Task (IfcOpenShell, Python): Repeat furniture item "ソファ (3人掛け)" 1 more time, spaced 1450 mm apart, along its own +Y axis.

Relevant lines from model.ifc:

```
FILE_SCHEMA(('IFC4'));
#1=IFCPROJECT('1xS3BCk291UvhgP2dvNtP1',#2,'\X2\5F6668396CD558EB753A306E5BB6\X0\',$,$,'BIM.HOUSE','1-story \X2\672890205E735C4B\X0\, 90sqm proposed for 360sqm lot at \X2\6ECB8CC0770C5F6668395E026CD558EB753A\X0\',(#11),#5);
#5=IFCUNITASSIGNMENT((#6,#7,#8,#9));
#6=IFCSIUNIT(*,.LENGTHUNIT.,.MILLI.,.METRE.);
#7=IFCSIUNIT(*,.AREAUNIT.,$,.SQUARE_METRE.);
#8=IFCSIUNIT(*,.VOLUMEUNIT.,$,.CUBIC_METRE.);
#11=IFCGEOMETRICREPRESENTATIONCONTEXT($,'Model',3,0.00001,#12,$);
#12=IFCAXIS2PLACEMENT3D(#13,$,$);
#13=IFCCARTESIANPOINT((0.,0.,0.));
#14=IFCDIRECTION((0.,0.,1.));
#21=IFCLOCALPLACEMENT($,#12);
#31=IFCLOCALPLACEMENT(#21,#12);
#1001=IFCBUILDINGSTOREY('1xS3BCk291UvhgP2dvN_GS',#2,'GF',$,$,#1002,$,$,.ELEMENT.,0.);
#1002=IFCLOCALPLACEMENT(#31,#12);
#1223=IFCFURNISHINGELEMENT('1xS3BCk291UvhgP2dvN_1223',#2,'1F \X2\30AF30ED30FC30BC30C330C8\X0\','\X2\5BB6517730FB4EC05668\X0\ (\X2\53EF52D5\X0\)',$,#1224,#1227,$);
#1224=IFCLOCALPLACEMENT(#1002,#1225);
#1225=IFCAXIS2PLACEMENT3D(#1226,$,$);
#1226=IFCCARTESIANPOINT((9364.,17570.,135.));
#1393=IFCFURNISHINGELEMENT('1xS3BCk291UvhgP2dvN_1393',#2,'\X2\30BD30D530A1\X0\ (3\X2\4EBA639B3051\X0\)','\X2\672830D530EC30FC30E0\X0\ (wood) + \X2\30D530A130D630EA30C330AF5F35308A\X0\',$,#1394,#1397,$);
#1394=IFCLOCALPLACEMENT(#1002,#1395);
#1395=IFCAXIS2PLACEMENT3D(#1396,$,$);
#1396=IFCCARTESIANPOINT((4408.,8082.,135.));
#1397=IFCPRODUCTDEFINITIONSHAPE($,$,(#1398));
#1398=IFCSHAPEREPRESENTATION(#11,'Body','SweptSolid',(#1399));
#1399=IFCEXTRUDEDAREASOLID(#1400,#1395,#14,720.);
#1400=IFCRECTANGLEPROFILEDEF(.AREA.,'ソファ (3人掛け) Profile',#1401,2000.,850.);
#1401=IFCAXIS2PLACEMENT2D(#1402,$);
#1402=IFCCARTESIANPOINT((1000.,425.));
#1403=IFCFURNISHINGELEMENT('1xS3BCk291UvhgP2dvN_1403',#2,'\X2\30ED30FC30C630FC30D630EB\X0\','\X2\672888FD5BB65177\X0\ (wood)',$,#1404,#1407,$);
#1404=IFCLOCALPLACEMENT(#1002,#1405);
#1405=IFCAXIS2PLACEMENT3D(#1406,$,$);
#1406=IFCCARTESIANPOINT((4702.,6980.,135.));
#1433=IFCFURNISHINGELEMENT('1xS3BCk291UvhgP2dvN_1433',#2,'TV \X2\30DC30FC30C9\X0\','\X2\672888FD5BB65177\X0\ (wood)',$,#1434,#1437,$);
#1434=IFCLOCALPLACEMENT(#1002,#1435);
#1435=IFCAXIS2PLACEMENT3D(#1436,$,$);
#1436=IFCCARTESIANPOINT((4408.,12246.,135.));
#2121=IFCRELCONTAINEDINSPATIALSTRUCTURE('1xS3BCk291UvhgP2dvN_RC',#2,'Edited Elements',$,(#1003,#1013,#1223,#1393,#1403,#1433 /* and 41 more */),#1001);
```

```python
import ifcopenshell
import ifcopenshell.api.geometry
import ifcopenshell.api.root
import ifcopenshell.util.element
import ifcopenshell.util.placement
import ifcopenshell.util.unit

model = ifcopenshell.open("model.ifc")
unit_scale = ifcopenshell.util.unit.calculate_unit_scale(model)


def reuse_history(source, copy):
    """copy_class also copies each property set's owner history, people and application; keep the originals."""
    for rel in copy.IsDefinedBy:
        if rel.is_a("IfcRelDefinesByProperties") and (history := rel.RelatingPropertyDefinition.OwnerHistory):
            rel.RelatingPropertyDefinition.OwnerHistory = source.OwnerHistory
            ifcopenshell.util.element.remove_deep2(model, history)


source = model.by_id(1393)
base = ifcopenshell.util.placement.get_local_placement(source.ObjectPlacement)
step = base[:3, 1] * 1.45 / unit_scale

for i in range(1, 2):
    copy = ifcopenshell.api.root.copy_class(model, product=source)
    copy.Representation = ifcopenshell.util.element.copy_deep(
        model, source.Representation, exclude=["IfcGeometricRepresentationContext", "IfcRepresentationMap"]
    )
    reuse_history(source, copy)
    matrix = base.copy()
    matrix[:3, 3] += i * step
    print("added at", matrix[:3, 3].round(3) + 0.0)
    ifcopenshell.api.geometry.edit_object_placement(model, product=copy, matrix=matrix, is_si=False)

model.write("model_updated.ifc")
```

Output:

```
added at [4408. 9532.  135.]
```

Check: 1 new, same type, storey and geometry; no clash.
